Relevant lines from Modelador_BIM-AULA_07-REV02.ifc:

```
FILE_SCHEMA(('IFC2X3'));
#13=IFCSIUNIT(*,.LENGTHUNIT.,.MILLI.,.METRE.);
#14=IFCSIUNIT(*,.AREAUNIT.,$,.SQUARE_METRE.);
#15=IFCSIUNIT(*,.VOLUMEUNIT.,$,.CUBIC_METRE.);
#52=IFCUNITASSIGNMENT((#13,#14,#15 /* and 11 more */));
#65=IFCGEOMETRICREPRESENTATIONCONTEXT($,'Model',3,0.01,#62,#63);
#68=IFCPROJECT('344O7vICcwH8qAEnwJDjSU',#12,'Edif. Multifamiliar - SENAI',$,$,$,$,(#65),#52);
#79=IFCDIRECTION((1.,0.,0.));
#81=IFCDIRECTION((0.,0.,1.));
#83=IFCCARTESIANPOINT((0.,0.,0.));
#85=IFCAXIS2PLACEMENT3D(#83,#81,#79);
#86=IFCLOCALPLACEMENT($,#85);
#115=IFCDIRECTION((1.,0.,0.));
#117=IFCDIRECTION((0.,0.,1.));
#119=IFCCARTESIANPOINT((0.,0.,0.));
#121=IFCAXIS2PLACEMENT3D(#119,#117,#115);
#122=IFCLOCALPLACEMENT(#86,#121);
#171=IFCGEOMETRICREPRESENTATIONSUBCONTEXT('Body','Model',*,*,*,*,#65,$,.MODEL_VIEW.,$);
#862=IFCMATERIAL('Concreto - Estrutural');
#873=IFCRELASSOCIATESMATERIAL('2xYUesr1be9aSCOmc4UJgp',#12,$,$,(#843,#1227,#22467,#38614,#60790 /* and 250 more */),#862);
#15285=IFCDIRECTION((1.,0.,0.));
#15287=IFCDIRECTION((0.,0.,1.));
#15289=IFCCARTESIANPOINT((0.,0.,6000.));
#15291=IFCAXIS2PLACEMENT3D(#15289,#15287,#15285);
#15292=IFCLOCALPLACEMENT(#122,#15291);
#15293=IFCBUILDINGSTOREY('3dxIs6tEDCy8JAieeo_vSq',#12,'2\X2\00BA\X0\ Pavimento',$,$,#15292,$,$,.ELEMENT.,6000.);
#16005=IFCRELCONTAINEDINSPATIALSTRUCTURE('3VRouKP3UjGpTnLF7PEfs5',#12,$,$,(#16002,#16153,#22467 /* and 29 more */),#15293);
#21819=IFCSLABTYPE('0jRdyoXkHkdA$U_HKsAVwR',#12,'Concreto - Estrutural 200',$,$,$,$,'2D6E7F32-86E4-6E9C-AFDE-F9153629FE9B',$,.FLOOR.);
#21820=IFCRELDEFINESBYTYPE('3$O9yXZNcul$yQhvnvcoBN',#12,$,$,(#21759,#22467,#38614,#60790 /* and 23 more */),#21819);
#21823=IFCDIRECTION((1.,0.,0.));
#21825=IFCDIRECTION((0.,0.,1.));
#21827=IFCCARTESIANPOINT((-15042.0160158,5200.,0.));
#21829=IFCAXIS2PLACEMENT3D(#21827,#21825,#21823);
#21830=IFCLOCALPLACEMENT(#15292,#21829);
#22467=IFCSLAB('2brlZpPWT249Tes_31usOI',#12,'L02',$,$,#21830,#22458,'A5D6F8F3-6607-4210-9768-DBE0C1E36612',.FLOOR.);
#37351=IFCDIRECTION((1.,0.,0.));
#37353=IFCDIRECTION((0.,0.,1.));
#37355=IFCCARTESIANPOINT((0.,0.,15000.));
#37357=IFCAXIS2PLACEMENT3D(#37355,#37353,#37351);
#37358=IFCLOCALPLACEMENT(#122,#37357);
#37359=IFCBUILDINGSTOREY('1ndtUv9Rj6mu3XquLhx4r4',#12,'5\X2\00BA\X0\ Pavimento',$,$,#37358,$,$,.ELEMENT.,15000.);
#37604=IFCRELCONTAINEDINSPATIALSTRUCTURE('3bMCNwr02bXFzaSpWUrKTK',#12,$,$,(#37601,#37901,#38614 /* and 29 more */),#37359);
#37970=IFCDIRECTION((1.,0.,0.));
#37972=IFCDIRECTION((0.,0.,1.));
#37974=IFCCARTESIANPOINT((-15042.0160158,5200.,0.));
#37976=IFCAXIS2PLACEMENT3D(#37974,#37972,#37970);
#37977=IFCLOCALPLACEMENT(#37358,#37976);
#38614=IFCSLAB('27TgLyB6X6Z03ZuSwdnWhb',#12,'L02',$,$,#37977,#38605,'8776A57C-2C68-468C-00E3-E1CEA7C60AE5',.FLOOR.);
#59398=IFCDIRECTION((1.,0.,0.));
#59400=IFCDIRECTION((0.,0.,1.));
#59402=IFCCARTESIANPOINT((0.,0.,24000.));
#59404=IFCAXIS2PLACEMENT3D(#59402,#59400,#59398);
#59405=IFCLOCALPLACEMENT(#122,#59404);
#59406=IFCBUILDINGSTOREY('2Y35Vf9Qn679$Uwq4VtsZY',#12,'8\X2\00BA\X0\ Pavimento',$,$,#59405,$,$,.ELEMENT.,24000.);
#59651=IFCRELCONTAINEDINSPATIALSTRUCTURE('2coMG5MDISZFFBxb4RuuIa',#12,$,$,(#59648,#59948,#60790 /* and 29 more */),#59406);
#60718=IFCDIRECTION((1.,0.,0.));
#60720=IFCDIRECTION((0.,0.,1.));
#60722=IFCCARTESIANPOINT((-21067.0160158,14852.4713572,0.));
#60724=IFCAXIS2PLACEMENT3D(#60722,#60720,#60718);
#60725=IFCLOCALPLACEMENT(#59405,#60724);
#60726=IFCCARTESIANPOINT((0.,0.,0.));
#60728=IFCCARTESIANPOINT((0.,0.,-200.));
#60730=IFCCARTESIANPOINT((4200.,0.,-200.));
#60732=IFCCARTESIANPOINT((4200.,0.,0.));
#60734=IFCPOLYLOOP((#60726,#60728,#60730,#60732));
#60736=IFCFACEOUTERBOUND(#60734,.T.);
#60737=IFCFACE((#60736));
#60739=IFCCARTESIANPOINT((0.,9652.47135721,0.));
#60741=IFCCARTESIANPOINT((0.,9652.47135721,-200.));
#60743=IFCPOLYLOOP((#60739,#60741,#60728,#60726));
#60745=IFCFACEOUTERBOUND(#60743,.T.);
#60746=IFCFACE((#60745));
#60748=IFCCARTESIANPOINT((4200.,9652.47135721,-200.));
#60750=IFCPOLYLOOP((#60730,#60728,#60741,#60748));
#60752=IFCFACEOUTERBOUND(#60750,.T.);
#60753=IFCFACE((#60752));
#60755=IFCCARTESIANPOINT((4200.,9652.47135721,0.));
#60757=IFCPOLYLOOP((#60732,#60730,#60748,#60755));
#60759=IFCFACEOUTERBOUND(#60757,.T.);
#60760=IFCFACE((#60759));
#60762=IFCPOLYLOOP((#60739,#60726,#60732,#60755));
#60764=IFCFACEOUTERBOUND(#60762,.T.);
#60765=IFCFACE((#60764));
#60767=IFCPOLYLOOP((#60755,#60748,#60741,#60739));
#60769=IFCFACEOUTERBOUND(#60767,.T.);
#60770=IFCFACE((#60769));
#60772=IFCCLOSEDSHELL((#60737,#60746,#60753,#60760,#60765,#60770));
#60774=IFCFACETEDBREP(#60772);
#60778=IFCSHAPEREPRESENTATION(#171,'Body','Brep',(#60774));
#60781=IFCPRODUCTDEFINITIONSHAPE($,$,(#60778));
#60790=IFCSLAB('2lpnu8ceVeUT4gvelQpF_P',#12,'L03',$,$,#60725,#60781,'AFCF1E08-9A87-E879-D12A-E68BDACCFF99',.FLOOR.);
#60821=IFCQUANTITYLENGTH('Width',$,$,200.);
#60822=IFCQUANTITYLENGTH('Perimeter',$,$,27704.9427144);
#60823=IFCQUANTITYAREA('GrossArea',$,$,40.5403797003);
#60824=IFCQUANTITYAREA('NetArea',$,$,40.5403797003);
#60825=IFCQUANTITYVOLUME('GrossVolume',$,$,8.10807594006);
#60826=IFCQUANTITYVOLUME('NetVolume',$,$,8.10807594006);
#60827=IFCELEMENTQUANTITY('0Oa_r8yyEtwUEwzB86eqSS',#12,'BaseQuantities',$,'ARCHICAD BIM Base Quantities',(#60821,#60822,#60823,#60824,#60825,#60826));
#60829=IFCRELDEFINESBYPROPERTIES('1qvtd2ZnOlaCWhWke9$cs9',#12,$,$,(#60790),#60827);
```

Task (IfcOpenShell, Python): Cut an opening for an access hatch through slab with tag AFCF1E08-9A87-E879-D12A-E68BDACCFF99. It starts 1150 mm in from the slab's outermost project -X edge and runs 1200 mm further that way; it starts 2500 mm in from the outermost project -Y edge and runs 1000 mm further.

```python
import numpy as np
import ifcopenshell
import ifcopenshell.api.feature
import ifcopenshell.api.geometry
import ifcopenshell.api.pset
import ifcopenshell.api.root
import ifcopenshell.geom
import ifcopenshell.util.element
import ifcopenshell.util.placement
import ifcopenshell.util.representation
import ifcopenshell.util.shape
import ifcopenshell.util.unit

model = ifcopenshell.open("Modelador_BIM-AULA_07-REV02.ifc")
unit_scale = ifcopenshell.util.unit.calculate_unit_scale(model)
area_scale = ifcopenshell.util.unit.calculate_unit_scale(model, "AREAUNIT")
volume_scale = ifcopenshell.util.unit.calculate_unit_scale(model, "VOLUMEUNIT")
settings = ifcopenshell.geom.settings()


def volume(element):
    """Net volume in cubic metres, openings subtracted."""
    shape = ifcopenshell.geom.create_shape(settings, element)
    return ifcopenshell.util.shape.get_volume(shape.geometry)


slab = model.by_guid("2lpnu8ceVeUT4gvelQpF_P")
before = volume(slab)

# Extent in the slab's own axes, in metres. The edges named are its -X and -Y sides.
slab_shape = ifcopenshell.geom.create_shape(settings, slab)
vertices = ifcopenshell.util.shape.get_vertices(slab_shape.geometry)
x_min, y_min, bottom = vertices.min(axis=0)
top = vertices[:, 2].max()

opening = ifcopenshell.api.root.create_entity(model, ifc_class="IfcOpeningElement", name="Access hatch opening")
context = ifcopenshell.util.representation.get_context(model, "Model", "Body", "MODEL_VIEW")
width, depth = 1.2, 1
outline = [(0.0, 0.0), (width, 0.0), (width, depth), (0.0, depth), (0.0, 0.0)]
# Overshoot both faces by 50 mm so the cut is clean.
shape = ifcopenshell.api.geometry.add_slab_representation(
    model, context=context, depth=top - bottom + 0.1, polyline=outline
)
ifcopenshell.api.geometry.assign_representation(model, product=opening, representation=shape)

matrix = ifcopenshell.util.placement.get_local_placement(slab.ObjectPlacement)
matrix[:, 3] = matrix @ np.append(np.array([x_min + 1.15, y_min + 2.5, bottom - 0.05]) / unit_scale, 1.0)
ifcopenshell.api.geometry.edit_object_placement(model, product=opening, matrix=matrix, is_si=False)
ifcopenshell.api.feature.add_feature(model, feature=opening, element=slab)

after = volume(slab)

# Update the slab's stored quantities.
qto = model.by_id(ifcopenshell.util.element.get_pset(slab, "BaseQuantities", should_inherit=False)["id"])
ifcopenshell.api.pset.edit_qto(model, qto=qto, properties={
    "NetArea": after / (top - bottom) / area_scale,
    "NetVolume": after / volume_scale,
})

print(f"slab volume {before:.3f} -> {after:.3f} m3")

model.write("Modelador_BIM-AULA_07-REV02_rev.ifc")
```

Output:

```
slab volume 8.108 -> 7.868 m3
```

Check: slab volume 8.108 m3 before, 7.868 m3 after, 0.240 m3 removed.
